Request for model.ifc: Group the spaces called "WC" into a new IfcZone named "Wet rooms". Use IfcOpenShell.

First a look at what the model holds.

```python
import ifcopenshell

model = ifcopenshell.open("model.ifc")
print(model.schema)
seen = {}
for space in model.by_type("IfcSpace"):
    seen[space.LongName] = seen.get(space.LongName, 0) + 1
for name, count in sorted(seen.items(), key=str):
    print(count, "x", name)
print("zones:", [z.Name for z in model.by_type("IfcZone")][:20])
```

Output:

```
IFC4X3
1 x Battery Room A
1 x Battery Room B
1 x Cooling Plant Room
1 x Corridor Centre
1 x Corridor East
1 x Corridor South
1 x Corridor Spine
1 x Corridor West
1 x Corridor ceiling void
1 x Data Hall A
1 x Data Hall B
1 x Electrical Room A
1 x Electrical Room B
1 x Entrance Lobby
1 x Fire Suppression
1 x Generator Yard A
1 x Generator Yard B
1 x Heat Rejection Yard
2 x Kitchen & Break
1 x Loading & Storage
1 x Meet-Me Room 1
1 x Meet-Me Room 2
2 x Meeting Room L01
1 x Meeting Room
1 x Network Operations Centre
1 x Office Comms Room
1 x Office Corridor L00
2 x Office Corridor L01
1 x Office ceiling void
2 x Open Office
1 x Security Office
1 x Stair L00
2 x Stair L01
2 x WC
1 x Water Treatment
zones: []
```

```python
import ifcopenshell
import ifcopenshell.api.group
import ifcopenshell.api.root

model = ifcopenshell.open("model.ifc")

names = {"WC"}
spaces = [s for s in model.by_type("IfcSpace") if s.LongName in names]

zone = ifcopenshell.api.root.create_entity(model, ifc_class="IfcZone", name="Wet rooms")
ifcopenshell.api.group.assign_group(model, products=spaces, group=zone)
print(len(spaces), "spaces in", zone.Name)

model.write("model_updated.ifc")
```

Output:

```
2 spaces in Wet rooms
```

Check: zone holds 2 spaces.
